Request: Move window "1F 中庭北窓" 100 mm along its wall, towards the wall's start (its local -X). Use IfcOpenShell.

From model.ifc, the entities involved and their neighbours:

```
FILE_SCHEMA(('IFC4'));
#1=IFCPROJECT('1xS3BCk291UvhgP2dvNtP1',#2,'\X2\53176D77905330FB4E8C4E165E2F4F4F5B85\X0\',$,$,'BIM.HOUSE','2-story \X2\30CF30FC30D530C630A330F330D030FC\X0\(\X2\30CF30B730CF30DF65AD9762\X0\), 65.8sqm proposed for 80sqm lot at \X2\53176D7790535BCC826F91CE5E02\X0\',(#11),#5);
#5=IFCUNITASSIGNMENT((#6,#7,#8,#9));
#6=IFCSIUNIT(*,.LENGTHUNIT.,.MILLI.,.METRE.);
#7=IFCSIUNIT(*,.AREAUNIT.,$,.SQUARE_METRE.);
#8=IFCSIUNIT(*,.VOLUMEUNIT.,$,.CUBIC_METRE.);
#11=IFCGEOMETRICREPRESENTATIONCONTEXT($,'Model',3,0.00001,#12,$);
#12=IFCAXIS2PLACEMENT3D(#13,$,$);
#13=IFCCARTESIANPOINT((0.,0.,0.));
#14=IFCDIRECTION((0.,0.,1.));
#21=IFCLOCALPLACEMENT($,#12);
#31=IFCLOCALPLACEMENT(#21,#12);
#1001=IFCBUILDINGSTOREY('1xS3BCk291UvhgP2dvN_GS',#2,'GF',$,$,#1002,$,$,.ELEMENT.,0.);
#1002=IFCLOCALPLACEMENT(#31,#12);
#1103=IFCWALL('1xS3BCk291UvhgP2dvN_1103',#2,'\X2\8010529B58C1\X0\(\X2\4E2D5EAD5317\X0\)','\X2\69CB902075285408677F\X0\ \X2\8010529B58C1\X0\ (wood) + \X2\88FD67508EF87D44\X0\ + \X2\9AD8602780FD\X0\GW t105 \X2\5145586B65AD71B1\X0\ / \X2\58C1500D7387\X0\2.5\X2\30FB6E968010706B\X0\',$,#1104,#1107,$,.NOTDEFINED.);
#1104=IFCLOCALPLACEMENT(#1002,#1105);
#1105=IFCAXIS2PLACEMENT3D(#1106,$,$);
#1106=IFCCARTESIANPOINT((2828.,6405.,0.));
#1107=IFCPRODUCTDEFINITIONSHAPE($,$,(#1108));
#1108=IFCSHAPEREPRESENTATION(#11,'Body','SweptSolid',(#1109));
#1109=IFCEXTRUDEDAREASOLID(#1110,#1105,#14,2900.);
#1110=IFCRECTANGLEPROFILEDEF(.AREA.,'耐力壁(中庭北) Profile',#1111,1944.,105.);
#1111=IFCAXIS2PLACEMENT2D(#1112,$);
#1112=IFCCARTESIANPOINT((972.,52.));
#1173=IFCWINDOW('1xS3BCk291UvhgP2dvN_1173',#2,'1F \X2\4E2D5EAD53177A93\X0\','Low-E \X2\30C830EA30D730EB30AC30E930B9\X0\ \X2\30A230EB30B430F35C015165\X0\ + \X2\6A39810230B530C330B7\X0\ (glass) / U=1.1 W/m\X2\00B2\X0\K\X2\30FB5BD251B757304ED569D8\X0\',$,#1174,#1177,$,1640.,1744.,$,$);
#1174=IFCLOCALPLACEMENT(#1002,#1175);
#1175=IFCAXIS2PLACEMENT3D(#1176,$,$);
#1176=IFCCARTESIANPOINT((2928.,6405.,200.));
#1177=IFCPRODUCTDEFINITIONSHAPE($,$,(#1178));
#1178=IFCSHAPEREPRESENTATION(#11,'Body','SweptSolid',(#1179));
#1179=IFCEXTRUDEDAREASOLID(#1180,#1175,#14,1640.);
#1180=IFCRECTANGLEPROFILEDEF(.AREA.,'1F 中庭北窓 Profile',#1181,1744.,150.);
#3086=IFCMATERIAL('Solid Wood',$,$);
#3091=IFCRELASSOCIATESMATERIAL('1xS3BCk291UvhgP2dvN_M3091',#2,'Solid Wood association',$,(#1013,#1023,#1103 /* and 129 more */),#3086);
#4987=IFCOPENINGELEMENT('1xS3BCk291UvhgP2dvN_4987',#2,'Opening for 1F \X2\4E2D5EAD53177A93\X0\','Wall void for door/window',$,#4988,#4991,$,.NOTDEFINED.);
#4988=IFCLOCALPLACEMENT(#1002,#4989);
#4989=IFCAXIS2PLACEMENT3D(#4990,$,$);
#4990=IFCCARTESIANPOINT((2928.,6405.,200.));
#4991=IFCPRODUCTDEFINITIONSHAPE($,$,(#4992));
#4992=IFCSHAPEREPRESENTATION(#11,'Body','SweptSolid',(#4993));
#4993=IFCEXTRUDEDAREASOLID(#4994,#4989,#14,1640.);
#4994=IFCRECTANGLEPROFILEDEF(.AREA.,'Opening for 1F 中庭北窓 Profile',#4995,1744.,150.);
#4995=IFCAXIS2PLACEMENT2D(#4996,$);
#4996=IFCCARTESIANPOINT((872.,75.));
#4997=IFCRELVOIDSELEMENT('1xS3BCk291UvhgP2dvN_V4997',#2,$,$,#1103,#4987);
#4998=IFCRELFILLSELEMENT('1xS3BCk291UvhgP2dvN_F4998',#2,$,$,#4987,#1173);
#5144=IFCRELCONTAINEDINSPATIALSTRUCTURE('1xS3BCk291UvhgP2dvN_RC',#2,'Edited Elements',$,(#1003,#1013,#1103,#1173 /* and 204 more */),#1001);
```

```python
import ifcopenshell
import ifcopenshell.api.geometry
import ifcopenshell.util.placement

model = ifcopenshell.open("model.ifc")

window = model.by_guid("1xS3BCk291UvhgP2dvN_1173")
opening = window.FillsVoids[0].RelatingOpeningElement
wall = opening.VoidsElements[0].RelatingBuildingElement

wall_matrix = ifcopenshell.util.placement.get_local_placement(wall.ObjectPlacement)
shift = wall_matrix[:3, 0] * -100.0
before = ifcopenshell.util.placement.get_local_placement(window.ObjectPlacement)[:3, 3].copy()

# The window is not placed relative to its opening, so move both.
for product in (opening, window):
    matrix = ifcopenshell.util.placement.get_local_placement(product.ObjectPlacement)
    matrix[:3, 3] += shift
    ifcopenshell.api.geometry.edit_object_placement(model, product=product, matrix=matrix, is_si=False)

after = ifcopenshell.util.placement.get_local_placement(window.ObjectPlacement)[:3, 3]
print("window moved by", (after - before).round(3) + 0.0)

model.write("model_rev.ifc")
```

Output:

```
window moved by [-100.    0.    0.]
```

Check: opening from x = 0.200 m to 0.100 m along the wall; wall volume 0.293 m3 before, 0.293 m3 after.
